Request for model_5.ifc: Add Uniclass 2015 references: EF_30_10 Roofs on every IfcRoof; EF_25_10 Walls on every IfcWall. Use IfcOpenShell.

First a look at what the model holds.

```python
import ifcopenshell

model = ifcopenshell.open("model_5.ifc")
print(model.schema)
print("classifications:", [c.Name for c in model.by_type("IfcClassification")])
for ifc_class in ("IfcDoor", "IfcRoof", "IfcStair", "IfcWall", "IfcWindow"):
    print(ifc_class, len(model.by_type(ifc_class)))
```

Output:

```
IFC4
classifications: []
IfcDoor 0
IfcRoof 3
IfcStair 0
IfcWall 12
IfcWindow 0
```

```python
import ifcopenshell
import ifcopenshell.api.classification

model = ifcopenshell.open("model_5.ifc")

system = ifcopenshell.api.classification.add_classification(model, classification="Uniclass 2015")

codes = {
    "IfcRoof": ("EF_30_10", "Roofs"),
    "IfcWall": ("EF_25_10", "Walls"),
}
for ifc_class, (code, name) in codes.items():
    products = model.by_type(ifc_class)
    ifcopenshell.api.classification.add_reference(
        model, products=products, classification=system, identification=code, name=name
    )
    print(code, len(products))

model.write("model_5_updated.ifc")
```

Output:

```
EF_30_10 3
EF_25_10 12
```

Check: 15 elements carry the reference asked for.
